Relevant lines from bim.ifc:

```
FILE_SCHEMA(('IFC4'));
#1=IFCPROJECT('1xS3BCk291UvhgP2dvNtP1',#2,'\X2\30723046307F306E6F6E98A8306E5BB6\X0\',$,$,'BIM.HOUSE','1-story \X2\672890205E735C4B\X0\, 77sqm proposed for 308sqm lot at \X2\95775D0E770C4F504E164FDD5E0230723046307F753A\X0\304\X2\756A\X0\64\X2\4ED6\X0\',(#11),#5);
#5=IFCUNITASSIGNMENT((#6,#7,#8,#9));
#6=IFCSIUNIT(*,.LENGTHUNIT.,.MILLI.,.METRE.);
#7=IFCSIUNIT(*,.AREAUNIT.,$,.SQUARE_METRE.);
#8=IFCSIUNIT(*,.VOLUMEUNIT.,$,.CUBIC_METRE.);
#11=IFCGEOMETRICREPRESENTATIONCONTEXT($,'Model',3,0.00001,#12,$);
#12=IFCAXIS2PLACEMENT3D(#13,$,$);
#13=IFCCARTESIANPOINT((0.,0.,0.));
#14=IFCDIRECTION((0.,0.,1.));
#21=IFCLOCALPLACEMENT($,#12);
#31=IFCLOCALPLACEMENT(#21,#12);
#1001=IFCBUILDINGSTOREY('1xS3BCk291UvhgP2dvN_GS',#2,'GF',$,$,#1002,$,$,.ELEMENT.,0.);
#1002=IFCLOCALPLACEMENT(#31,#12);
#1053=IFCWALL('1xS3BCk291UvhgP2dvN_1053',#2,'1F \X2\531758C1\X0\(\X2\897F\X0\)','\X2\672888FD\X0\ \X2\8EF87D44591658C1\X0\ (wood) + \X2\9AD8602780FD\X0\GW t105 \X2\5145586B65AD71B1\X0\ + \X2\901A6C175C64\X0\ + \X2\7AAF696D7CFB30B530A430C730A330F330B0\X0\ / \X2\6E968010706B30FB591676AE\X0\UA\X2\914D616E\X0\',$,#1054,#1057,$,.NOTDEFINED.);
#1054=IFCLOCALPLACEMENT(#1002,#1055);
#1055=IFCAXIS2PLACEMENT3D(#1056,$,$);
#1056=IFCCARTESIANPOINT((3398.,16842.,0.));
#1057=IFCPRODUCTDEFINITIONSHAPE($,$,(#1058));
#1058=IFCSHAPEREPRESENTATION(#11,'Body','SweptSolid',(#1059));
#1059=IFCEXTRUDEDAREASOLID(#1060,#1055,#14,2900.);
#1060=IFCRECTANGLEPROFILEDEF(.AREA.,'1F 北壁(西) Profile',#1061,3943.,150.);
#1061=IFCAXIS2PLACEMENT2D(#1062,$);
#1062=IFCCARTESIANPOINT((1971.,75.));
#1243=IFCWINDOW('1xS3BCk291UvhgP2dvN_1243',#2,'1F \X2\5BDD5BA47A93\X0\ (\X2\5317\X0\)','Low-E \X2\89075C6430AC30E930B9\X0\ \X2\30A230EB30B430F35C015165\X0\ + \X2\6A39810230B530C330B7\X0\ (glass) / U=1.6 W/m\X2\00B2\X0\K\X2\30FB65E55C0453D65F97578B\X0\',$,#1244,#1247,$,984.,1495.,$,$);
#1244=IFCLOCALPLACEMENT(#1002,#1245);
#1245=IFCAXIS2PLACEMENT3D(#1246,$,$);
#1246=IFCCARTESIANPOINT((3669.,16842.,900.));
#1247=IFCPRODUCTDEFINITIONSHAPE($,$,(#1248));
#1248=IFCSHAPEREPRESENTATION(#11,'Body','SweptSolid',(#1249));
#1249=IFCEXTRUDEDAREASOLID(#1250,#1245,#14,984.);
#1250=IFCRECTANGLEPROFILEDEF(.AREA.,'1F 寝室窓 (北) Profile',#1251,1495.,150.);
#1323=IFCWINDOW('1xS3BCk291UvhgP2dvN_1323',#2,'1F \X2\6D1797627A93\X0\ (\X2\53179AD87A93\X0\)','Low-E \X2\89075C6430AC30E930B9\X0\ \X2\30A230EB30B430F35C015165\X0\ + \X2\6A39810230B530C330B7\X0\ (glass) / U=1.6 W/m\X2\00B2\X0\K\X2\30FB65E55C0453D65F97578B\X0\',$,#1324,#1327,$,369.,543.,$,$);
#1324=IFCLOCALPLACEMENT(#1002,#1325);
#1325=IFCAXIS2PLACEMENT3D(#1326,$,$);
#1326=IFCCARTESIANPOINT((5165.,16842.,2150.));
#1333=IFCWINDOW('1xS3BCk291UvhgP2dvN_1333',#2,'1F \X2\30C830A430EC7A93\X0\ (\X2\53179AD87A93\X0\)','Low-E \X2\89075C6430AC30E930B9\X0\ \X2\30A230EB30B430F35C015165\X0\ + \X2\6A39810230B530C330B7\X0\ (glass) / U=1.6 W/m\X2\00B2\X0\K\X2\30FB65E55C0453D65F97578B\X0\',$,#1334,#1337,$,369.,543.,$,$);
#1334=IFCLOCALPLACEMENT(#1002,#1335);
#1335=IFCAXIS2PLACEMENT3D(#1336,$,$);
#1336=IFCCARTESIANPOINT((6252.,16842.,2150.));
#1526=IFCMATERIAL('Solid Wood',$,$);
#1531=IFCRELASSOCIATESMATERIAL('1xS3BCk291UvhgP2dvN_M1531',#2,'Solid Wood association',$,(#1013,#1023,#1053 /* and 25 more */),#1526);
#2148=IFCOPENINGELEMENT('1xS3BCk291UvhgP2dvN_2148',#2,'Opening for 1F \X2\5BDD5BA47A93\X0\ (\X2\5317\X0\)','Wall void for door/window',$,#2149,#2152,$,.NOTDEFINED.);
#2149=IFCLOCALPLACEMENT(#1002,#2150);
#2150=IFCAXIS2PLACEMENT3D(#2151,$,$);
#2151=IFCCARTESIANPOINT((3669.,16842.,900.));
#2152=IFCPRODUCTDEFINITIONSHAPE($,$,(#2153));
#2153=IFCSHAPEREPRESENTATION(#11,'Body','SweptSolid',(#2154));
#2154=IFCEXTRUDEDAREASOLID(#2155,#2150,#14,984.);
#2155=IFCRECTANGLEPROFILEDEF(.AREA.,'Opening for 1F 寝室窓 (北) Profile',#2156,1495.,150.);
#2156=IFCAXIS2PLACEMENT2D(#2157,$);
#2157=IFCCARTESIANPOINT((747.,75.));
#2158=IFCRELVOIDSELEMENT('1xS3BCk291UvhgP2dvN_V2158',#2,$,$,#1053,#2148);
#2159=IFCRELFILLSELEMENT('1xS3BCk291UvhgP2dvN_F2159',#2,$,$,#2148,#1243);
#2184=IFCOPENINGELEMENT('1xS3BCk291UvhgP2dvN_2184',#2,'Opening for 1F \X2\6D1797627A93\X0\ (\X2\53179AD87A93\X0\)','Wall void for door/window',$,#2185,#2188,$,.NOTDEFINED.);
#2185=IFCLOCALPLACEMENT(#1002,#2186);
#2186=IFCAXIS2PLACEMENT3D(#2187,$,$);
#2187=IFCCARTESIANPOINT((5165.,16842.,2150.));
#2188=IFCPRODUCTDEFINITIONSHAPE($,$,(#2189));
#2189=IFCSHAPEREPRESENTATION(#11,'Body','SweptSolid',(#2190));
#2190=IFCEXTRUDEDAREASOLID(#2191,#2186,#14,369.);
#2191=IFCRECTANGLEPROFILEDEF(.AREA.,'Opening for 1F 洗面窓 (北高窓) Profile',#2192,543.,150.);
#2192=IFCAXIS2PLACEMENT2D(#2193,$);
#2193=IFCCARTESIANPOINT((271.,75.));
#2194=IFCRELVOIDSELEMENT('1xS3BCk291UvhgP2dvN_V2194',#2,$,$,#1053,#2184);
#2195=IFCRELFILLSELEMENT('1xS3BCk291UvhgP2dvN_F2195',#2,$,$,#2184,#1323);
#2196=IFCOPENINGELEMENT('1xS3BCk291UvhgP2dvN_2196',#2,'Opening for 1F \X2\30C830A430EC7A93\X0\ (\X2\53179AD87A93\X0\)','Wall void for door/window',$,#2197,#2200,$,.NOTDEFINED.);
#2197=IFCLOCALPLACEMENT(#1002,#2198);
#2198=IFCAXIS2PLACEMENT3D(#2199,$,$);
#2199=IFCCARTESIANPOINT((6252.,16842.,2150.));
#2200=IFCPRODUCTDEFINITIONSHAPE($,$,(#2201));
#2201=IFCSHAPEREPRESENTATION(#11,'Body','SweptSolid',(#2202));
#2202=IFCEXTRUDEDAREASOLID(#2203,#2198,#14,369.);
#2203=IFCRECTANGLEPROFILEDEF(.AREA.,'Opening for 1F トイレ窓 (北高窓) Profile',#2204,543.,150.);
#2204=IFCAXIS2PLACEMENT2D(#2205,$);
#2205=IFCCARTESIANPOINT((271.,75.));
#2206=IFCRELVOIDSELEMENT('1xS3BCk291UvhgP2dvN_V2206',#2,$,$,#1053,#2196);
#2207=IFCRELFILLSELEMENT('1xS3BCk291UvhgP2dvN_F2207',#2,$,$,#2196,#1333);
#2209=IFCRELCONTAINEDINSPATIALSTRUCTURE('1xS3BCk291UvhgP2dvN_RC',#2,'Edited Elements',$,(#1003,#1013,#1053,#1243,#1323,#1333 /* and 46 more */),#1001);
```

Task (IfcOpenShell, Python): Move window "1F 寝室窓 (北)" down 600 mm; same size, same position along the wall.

```python
import numpy as np
import ifcopenshell
import ifcopenshell.api.geometry
import ifcopenshell.util.placement
import ifcopenshell.util.unit

model = ifcopenshell.open("bim.ifc")
unit_scale = ifcopenshell.util.unit.calculate_unit_scale(model)

window = model.by_guid("1xS3BCk291UvhgP2dvN_1243")
opening = window.FillsVoids[0].RelatingOpeningElement
dz = -0.6 / unit_scale

shift = np.array([0.0, 0.0, dz])
# The window is not placed relative to its opening, so move both.
for product in (opening, window):
    matrix = ifcopenshell.util.placement.get_local_placement(product.ObjectPlacement)
    matrix[:3, 3] += shift
    ifcopenshell.api.geometry.edit_object_placement(model, product=product, matrix=matrix, is_si=False)

print(f"moved by {dz * unit_scale:+.3f} m")

model.write("bim_rev.ifc")
```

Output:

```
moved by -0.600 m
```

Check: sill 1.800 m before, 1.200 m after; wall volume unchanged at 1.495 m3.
